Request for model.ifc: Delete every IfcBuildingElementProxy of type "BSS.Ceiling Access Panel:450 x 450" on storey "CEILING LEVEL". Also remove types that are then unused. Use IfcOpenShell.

First a look at what the model holds.

```python
import ifcopenshell
import ifcopenshell.util.element

model = ifcopenshell.open("model.ifc")
print(model.schema)
storey = next(s for s in model.by_type("IfcBuildingStorey") if s.Name == "CEILING LEVEL")
proxies = [e for e in ifcopenshell.util.element.get_decomposition(storey) if e.is_a("IfcBuildingElementProxy")]
seen = {}
for e in proxies:
    element_type = ifcopenshell.util.element.get_type(e)
    name = element_type.Name if element_type not in (None, e) else None
    seen[name] = seen.get(name, 0) + 1
for name, count in sorted(seen.items(), key=str):
    print(count, "x", name)
```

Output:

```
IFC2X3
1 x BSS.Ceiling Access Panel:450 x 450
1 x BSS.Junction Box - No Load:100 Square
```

```python
import ifcopenshell
import ifcopenshell.api.root
import ifcopenshell.util.element

model = ifcopenshell.open("model.ifc")

storey = next(s for s in model.by_type("IfcBuildingStorey") if s.Name == "CEILING LEVEL")
proxies = [e for e in ifcopenshell.util.element.get_decomposition(storey) if e.is_a("IfcBuildingElementProxy")]
targets = [e for e in proxies if (t := ifcopenshell.util.element.get_type(e)) not in (None, e) and t.Name == "BSS.Ceiling Access Panel:450 x 450"]
types = {ifcopenshell.util.element.get_type(e) for e in targets} - {None, *targets}

for e in targets:
    ifcopenshell.api.root.remove_product(model, product=e)
print(len(targets), "removed")

unused = [t for t in types if not ifcopenshell.util.element.get_types(t)]
for t in unused:
    ifcopenshell.api.root.remove_product(model, product=t)
print(len(unused), "unused types removed")

model.write("model_edited.ifc")
```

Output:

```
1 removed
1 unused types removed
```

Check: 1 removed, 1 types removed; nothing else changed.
